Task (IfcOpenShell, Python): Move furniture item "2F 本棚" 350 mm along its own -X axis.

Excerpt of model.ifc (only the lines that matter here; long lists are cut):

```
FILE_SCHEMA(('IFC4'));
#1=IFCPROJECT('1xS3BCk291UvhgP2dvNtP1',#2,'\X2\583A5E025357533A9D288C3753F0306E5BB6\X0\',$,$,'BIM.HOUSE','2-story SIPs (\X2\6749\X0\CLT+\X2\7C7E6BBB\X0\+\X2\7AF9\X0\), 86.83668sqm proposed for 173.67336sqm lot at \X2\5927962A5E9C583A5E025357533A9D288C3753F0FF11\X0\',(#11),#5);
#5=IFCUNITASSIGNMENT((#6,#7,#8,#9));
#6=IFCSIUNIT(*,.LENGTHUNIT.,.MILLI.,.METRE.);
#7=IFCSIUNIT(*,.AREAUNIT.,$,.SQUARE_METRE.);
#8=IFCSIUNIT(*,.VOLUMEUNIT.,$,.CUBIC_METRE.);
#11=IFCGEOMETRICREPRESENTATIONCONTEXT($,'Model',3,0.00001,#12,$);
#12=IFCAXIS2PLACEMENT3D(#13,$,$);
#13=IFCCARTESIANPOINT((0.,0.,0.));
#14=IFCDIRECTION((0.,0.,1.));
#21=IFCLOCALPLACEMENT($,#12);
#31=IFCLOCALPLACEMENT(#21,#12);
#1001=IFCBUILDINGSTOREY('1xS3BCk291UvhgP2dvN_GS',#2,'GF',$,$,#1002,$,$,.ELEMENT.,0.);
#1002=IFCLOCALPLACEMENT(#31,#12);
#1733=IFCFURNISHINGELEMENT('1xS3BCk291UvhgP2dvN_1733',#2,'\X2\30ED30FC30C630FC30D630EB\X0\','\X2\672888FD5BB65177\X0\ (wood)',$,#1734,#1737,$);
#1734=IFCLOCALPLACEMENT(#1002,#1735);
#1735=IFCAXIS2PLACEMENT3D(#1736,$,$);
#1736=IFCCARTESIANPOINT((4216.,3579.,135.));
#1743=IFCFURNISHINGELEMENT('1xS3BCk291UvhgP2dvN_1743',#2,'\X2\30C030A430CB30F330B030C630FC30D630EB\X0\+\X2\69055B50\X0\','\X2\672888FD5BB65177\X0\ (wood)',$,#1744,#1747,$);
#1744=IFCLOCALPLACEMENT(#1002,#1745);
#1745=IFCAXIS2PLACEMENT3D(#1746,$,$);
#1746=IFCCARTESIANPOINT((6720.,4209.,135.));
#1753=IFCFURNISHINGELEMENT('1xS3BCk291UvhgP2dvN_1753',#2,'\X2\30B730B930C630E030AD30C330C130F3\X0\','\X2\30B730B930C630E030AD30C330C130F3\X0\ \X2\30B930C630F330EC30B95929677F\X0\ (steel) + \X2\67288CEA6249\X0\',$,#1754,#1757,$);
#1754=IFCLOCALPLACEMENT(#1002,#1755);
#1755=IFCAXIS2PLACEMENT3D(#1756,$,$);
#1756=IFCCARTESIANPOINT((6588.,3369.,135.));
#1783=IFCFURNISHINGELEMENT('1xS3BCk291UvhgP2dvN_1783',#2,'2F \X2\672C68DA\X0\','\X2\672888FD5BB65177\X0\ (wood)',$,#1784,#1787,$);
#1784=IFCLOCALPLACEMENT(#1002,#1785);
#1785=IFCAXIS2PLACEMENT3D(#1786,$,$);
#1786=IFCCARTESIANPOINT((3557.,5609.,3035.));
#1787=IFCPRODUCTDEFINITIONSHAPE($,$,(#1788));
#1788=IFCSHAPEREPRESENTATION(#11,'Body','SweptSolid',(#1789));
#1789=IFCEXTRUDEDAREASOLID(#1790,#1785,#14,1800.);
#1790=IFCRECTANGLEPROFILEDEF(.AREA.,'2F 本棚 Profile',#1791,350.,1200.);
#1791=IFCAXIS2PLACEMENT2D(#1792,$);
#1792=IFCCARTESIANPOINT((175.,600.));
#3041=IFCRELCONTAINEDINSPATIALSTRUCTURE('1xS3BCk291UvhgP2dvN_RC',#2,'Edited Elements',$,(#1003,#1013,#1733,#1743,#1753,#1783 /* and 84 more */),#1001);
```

```python
import ifcopenshell
import ifcopenshell.api.geometry
import ifcopenshell.util.placement
import ifcopenshell.util.unit

model = ifcopenshell.open("model.ifc")
unit_scale = ifcopenshell.util.unit.calculate_unit_scale(model)

item = model.by_guid("1xS3BCk291UvhgP2dvN_1783")
matrix = ifcopenshell.util.placement.get_local_placement(item.ObjectPlacement)
matrix[:3, 3] -= matrix[:3, 0] * 0.35 / unit_scale
ifcopenshell.api.geometry.edit_object_placement(model, product=item, matrix=matrix, is_si=False)

print(ifcopenshell.util.placement.get_local_placement(item.ObjectPlacement).round(3) + 0.0)

model.write("model_updated.ifc")
```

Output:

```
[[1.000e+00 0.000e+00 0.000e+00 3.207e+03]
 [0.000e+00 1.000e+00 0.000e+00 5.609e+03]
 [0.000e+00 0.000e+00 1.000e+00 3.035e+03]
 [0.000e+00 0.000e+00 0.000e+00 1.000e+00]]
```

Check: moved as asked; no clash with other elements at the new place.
